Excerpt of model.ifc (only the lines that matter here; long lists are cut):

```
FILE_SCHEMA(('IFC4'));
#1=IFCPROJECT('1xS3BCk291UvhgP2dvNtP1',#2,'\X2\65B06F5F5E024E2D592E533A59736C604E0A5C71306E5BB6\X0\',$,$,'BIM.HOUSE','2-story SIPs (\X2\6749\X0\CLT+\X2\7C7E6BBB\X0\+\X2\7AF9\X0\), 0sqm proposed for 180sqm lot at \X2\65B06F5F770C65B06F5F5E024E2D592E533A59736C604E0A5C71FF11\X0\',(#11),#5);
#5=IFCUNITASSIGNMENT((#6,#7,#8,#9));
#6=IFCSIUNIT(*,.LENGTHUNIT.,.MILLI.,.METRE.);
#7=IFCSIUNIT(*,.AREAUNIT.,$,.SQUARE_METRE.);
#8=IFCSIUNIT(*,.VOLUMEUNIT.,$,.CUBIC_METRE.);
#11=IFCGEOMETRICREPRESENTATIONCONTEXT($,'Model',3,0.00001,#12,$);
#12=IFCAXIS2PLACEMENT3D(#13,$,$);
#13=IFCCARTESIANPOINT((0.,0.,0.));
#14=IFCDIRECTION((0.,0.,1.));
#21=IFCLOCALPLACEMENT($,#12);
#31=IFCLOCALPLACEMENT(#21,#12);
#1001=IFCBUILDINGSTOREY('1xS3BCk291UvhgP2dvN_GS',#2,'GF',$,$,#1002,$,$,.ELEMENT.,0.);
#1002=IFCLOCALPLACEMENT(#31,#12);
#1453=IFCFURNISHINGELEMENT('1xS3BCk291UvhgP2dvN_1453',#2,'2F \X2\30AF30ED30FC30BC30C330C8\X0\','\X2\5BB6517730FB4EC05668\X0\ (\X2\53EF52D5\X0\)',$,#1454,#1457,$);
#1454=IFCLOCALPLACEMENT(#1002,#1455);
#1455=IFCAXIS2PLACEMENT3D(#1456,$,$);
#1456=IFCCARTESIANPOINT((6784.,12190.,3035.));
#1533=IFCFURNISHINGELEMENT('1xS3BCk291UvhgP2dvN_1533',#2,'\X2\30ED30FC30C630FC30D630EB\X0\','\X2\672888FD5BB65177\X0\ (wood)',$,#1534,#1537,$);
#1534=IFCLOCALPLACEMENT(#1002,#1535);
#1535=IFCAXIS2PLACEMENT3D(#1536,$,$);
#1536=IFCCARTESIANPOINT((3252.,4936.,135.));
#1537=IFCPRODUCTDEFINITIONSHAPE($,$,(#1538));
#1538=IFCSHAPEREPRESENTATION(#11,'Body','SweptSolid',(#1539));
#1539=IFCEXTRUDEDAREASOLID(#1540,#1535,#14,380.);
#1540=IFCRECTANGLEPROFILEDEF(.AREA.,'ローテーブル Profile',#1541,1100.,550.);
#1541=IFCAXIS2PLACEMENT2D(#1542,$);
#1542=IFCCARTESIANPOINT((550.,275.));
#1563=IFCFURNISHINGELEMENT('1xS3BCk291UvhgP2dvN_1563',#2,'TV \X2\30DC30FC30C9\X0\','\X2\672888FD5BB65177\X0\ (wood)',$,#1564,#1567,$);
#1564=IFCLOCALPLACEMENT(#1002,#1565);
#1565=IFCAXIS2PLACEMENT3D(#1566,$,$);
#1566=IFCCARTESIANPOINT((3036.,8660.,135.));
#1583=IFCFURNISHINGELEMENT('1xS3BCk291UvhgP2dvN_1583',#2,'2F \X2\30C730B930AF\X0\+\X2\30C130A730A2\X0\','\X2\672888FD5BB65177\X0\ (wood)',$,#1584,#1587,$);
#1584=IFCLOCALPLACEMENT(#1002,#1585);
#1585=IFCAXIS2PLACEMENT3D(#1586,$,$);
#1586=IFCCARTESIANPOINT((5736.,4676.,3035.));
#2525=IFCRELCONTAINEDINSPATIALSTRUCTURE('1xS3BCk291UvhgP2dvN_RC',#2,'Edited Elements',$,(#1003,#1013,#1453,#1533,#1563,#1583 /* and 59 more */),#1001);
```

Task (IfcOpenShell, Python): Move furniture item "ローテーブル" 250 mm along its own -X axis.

```python
import ifcopenshell
import ifcopenshell.api.geometry
import ifcopenshell.util.placement
import ifcopenshell.util.unit

model = ifcopenshell.open("model.ifc")
unit_scale = ifcopenshell.util.unit.calculate_unit_scale(model)

item = model.by_id(1533)
matrix = ifcopenshell.util.placement.get_local_placement(item.ObjectPlacement)
matrix[:3, 3] -= matrix[:3, 0] * 0.25 / unit_scale
ifcopenshell.api.geometry.edit_object_placement(model, product=item, matrix=matrix, is_si=False)

print(ifcopenshell.util.placement.get_local_placement(item.ObjectPlacement).round(3) + 0.0)

model.write("model_v2.ifc")
```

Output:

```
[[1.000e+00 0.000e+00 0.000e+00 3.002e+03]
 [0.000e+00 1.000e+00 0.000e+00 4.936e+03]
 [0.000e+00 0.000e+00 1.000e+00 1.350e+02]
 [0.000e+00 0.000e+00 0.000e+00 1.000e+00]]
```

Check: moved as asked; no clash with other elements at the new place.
